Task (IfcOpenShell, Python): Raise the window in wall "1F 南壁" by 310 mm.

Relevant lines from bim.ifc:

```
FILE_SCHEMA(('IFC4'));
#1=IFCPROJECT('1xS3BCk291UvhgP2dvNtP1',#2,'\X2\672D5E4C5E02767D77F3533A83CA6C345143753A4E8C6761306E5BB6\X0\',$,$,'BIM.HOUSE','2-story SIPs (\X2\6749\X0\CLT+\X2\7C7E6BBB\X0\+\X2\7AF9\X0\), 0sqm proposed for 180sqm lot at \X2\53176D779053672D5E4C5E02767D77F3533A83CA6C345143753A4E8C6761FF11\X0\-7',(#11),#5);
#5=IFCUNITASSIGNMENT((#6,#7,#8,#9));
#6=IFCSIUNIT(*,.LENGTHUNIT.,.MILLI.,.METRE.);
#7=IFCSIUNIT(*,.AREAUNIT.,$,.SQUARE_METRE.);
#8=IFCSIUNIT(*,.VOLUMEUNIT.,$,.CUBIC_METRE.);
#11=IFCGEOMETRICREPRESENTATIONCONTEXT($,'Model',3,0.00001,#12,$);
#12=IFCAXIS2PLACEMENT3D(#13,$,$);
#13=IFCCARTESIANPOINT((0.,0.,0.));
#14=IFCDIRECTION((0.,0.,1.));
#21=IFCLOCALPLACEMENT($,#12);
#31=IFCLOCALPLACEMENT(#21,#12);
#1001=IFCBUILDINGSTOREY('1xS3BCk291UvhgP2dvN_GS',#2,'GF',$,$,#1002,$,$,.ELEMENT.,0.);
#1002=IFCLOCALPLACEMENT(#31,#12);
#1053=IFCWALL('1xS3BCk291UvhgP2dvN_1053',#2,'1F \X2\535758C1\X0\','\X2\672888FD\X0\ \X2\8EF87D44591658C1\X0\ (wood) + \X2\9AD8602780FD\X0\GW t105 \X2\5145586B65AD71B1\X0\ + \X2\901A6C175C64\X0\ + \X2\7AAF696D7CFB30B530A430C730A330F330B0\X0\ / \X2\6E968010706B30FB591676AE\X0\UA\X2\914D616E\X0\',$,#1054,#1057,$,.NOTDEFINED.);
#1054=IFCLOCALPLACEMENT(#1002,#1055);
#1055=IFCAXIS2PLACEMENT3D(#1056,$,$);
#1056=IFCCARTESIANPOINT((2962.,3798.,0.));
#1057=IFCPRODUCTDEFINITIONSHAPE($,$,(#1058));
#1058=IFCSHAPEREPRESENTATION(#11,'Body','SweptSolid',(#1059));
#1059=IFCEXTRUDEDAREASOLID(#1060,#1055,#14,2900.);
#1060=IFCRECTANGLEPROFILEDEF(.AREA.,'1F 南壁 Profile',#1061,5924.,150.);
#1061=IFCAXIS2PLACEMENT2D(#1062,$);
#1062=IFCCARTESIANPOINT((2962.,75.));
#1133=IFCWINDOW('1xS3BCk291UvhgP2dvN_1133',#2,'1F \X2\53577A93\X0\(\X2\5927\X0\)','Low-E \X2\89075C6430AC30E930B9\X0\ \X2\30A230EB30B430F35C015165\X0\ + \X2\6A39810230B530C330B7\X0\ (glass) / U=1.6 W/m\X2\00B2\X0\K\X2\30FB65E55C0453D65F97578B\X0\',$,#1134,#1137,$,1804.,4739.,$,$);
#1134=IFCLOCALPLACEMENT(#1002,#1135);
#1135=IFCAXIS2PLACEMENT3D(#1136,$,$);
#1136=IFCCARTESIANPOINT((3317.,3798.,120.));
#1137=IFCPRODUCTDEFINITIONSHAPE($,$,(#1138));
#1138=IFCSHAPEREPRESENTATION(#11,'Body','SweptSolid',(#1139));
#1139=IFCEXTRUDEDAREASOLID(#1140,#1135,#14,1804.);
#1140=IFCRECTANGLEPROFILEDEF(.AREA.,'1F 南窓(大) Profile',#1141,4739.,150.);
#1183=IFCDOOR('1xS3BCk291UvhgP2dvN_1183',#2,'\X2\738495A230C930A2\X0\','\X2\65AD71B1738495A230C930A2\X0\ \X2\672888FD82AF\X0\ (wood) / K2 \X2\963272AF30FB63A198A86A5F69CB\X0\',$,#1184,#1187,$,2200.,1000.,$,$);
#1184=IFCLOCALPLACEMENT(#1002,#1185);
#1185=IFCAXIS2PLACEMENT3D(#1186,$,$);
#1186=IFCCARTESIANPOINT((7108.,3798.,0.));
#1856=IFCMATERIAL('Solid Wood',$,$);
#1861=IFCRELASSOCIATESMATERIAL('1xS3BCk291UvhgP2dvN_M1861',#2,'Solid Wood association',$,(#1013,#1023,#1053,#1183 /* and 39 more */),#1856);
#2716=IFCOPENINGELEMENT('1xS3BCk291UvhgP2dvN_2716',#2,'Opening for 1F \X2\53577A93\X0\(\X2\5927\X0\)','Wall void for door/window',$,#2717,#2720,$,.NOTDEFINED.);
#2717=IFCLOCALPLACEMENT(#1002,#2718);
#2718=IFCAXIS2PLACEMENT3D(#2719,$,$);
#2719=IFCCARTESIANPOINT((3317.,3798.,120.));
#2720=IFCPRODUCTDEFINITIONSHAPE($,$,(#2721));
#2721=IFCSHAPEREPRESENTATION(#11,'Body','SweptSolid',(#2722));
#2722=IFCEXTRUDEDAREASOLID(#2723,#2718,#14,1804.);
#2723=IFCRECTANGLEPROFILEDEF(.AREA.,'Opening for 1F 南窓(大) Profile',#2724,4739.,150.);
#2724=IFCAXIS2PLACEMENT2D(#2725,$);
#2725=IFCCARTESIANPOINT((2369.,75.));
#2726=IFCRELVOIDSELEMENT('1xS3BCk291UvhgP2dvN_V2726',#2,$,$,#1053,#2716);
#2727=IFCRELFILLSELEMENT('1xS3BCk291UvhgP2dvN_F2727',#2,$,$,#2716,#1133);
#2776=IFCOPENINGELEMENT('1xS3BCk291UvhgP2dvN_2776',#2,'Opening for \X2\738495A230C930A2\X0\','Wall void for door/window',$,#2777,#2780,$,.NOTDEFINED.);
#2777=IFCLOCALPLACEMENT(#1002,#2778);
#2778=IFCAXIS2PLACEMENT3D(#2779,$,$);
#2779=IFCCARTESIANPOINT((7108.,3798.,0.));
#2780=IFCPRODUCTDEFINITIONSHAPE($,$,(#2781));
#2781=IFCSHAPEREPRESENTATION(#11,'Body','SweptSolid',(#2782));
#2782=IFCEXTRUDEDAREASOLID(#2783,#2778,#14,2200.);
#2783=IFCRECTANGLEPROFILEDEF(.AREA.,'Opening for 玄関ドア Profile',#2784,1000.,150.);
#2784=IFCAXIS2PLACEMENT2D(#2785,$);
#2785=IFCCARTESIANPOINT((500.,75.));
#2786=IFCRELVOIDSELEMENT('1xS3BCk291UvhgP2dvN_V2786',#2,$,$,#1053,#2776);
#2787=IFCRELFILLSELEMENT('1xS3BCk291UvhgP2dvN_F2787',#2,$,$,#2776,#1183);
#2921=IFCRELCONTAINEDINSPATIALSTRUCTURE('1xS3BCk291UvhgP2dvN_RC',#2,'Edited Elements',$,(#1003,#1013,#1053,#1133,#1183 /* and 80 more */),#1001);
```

```python
import numpy as np
import ifcopenshell
import ifcopenshell.api.geometry
import ifcopenshell.util.placement
import ifcopenshell.util.unit

model = ifcopenshell.open("bim.ifc")
unit_scale = ifcopenshell.util.unit.calculate_unit_scale(model)

window = model.by_id(1133)
opening = window.FillsVoids[0].RelatingOpeningElement
dz = 310.0

shift = np.array([0.0, 0.0, dz])
# The window is not placed relative to its opening, so move both.
for product in (opening, window):
    matrix = ifcopenshell.util.placement.get_local_placement(product.ObjectPlacement)
    matrix[:3, 3] += shift
    ifcopenshell.api.geometry.edit_object_placement(model, product=product, matrix=matrix, is_si=False)

print(f"moved by {dz * unit_scale:+.3f} m")

model.write("bim-out.ifc")
```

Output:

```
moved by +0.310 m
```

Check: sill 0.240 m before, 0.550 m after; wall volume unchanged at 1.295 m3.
